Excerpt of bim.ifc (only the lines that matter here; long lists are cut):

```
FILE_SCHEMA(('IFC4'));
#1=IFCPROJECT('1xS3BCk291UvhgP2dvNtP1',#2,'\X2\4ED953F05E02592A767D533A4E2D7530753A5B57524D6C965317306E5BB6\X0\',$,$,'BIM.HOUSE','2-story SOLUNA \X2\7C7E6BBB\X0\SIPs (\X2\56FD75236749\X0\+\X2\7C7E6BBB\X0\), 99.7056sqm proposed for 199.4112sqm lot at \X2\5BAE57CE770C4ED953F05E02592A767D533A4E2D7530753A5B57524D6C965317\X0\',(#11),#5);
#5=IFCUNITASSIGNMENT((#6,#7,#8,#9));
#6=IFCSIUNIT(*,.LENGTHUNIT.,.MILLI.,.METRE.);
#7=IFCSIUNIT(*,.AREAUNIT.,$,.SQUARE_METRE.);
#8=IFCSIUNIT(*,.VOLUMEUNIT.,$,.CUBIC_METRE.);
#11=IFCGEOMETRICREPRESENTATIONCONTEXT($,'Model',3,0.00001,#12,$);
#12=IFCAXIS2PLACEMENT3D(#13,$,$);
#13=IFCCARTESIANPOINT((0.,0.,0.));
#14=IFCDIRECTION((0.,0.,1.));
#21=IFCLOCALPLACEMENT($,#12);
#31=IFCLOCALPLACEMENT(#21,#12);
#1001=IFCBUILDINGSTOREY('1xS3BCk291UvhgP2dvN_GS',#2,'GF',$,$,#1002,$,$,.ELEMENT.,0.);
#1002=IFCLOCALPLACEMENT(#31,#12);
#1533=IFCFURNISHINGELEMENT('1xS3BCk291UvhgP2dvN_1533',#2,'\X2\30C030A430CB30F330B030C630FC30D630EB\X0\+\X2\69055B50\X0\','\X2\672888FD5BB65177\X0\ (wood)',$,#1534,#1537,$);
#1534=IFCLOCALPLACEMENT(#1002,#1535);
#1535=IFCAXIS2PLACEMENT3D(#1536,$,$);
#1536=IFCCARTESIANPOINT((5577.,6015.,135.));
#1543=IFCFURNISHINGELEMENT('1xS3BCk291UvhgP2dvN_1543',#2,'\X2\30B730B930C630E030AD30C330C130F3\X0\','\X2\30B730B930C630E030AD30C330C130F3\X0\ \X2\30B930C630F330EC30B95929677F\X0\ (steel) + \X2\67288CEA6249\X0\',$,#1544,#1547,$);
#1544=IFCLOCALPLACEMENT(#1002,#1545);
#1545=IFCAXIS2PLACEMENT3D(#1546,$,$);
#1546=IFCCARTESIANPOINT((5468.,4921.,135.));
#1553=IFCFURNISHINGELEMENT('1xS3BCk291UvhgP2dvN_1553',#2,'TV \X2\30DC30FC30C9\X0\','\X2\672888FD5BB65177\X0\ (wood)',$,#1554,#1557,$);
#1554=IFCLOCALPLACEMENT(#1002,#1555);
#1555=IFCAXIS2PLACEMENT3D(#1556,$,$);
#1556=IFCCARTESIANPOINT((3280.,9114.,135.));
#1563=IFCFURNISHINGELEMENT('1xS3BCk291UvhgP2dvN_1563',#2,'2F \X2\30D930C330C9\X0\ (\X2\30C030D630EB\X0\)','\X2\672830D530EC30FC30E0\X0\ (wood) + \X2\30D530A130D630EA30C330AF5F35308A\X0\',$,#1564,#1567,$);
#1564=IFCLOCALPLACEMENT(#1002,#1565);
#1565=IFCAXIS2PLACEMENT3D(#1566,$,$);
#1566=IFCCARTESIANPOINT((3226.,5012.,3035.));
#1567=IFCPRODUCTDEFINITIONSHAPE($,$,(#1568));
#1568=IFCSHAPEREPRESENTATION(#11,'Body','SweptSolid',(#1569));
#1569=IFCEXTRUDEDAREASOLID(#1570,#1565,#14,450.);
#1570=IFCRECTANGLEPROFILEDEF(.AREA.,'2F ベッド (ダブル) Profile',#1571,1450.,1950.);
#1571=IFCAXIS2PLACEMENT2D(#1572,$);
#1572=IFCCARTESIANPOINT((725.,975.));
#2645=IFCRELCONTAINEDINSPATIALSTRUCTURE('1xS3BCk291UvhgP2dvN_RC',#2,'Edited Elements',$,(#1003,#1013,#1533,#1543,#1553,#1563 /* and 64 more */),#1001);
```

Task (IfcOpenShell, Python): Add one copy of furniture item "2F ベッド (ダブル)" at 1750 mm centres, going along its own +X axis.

```python
import ifcopenshell
import ifcopenshell.api.geometry
import ifcopenshell.api.root
import ifcopenshell.util.element
import ifcopenshell.util.placement
import ifcopenshell.util.unit

model = ifcopenshell.open("bim.ifc")
unit_scale = ifcopenshell.util.unit.calculate_unit_scale(model)


def reuse_history(source, copy):
    """copy_class also copies each property set's owner history, people and application; keep the originals."""
    for rel in copy.IsDefinedBy:
        if rel.is_a("IfcRelDefinesByProperties") and (history := rel.RelatingPropertyDefinition.OwnerHistory):
            rel.RelatingPropertyDefinition.OwnerHistory = source.OwnerHistory
            ifcopenshell.util.element.remove_deep2(model, history)


source = model.by_id(1563)
base = ifcopenshell.util.placement.get_local_placement(source.ObjectPlacement)
step = base[:3, 0] * 1.75 / unit_scale

for i in range(1, 2):
    copy = ifcopenshell.api.root.copy_class(model, product=source)
    copy.Representation = ifcopenshell.util.element.copy_deep(
        model, source.Representation, exclude=["IfcGeometricRepresentationContext", "IfcRepresentationMap"]
    )
    reuse_history(source, copy)
    matrix = base.copy()
    matrix[:3, 3] += i * step
    print("added at", matrix[:3, 3].round(3) + 0.0)
    ifcopenshell.api.geometry.edit_object_placement(model, product=copy, matrix=matrix, is_si=False)

model.write("bim_rev.ifc")
```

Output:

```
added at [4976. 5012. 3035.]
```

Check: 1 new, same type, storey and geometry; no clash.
